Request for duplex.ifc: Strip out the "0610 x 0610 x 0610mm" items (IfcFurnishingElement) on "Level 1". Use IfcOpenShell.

First a look at what the model holds.

```python
import ifcopenshell
import ifcopenshell.util.element

model = ifcopenshell.open("duplex.ifc")
print(model.schema)
storey = next(s for s in model.by_type("IfcBuildingStorey") if s.Name == "Level 1")
furniture = [e for e in ifcopenshell.util.element.get_decomposition(storey) if e.is_a("IfcFurnishingElement")]
seen = {}
for e in furniture:
    element_type = ifcopenshell.util.element.get_type(e)
    name = element_type.Name if element_type not in (None, e) else None
    seen[name] = seen.get(name, 0) + 1
for name, count in sorted(seen.items(), key=str):
    print(count, "x", name)
```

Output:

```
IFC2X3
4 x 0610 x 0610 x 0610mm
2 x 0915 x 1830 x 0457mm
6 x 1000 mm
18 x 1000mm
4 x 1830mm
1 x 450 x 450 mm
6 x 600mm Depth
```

```python
import ifcopenshell
import ifcopenshell.api.root
import ifcopenshell.util.element

model = ifcopenshell.open("duplex.ifc")

storey = next(s for s in model.by_type("IfcBuildingStorey") if s.Name == "Level 1")
furniture = [e for e in ifcopenshell.util.element.get_decomposition(storey) if e.is_a("IfcFurnishingElement")]
targets = [e for e in furniture if (t := ifcopenshell.util.element.get_type(e)) not in (None, e) and t.Name == "0610 x 0610 x 0610mm"]

for e in targets:
    ifcopenshell.api.root.remove_product(model, product=e)
print(len(targets), "removed")

model.write("duplex_updated.ifc")
```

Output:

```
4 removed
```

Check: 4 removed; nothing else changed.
